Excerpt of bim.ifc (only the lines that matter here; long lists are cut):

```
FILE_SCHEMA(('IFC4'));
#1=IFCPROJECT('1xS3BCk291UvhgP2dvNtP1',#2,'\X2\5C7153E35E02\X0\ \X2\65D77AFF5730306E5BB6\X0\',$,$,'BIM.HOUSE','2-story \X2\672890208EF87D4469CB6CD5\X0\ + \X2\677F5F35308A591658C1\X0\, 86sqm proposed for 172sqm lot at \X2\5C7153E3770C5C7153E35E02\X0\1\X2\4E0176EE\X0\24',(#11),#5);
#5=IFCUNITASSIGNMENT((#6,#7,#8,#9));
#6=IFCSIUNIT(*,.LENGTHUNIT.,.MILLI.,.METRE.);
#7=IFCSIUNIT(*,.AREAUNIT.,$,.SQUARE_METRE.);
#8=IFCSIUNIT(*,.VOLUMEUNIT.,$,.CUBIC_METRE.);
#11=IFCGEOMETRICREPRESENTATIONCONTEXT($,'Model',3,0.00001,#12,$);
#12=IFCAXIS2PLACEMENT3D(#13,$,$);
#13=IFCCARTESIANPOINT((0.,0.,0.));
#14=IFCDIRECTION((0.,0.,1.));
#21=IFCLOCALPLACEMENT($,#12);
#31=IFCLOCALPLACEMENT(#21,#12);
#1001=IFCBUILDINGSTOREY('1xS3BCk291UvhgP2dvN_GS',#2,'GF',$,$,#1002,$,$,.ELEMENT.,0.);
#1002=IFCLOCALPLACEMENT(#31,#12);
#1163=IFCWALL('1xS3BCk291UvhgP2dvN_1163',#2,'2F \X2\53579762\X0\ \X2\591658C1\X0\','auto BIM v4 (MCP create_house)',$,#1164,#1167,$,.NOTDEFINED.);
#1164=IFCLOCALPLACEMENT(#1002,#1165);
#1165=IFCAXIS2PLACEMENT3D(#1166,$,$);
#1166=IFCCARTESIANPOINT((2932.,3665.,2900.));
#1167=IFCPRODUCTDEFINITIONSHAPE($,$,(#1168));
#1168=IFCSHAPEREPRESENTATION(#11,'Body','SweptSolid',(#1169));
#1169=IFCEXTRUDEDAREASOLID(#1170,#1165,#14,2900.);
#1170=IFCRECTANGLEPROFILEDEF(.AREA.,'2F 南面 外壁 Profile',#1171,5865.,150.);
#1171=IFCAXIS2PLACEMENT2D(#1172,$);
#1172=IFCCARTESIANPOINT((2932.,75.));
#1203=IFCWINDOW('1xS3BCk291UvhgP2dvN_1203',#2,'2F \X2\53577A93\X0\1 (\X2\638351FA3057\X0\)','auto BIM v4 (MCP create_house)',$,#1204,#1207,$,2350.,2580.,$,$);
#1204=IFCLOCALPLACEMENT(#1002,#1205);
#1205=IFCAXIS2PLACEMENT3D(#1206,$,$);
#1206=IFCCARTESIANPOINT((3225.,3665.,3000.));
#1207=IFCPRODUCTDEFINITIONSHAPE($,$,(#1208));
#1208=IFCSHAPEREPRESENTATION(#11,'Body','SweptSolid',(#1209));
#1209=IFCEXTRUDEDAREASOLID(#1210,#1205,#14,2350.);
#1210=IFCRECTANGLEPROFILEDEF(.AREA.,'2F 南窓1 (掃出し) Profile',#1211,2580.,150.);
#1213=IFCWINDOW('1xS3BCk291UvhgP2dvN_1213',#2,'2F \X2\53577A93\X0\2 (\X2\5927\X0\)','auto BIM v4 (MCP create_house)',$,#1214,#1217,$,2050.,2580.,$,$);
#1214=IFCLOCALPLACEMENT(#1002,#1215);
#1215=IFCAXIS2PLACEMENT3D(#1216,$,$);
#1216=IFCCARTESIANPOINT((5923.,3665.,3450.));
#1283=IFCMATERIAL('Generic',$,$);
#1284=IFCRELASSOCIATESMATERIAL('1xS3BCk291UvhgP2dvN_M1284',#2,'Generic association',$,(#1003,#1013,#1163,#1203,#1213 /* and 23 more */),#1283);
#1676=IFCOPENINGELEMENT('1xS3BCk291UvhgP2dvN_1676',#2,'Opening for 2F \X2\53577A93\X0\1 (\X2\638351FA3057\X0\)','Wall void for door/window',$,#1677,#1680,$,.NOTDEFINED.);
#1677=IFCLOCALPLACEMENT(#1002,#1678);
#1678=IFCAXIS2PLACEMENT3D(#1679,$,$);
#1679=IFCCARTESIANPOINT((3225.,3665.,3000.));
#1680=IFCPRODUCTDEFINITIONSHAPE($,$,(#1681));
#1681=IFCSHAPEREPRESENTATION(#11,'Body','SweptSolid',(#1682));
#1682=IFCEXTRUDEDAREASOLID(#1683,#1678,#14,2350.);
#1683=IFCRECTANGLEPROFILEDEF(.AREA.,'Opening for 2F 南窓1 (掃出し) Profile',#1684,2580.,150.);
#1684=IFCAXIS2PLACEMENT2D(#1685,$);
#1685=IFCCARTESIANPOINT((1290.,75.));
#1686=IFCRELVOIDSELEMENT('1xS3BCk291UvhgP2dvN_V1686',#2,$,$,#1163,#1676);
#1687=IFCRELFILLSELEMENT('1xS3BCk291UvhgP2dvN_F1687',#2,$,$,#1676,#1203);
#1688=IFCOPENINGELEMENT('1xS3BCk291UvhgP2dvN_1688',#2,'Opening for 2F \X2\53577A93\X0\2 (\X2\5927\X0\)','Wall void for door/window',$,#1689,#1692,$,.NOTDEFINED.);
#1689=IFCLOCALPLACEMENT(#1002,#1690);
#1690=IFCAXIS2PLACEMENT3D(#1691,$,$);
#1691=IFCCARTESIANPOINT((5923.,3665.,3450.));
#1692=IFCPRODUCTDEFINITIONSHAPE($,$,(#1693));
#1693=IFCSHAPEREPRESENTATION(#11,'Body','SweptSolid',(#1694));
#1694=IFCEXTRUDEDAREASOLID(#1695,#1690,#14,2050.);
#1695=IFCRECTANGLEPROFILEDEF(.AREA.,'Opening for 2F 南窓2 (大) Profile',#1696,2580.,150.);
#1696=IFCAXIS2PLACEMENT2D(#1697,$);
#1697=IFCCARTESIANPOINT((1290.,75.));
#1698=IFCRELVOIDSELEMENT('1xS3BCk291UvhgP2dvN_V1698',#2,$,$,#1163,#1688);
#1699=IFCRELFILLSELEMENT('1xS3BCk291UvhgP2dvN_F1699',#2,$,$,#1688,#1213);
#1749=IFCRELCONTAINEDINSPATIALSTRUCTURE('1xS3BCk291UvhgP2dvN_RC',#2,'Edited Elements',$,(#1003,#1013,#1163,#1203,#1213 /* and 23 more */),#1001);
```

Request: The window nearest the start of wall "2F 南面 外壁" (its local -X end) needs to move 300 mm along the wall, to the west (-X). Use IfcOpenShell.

```python
import ifcopenshell
import ifcopenshell.api.geometry
import ifcopenshell.util.placement
import ifcopenshell.util.unit

model = ifcopenshell.open("bim.ifc")
unit_scale = ifcopenshell.util.unit.calculate_unit_scale(model)

window = model.by_guid("1xS3BCk291UvhgP2dvN_1203")
opening = window.FillsVoids[0].RelatingOpeningElement
wall = opening.VoidsElements[0].RelatingBuildingElement

wall_matrix = ifcopenshell.util.placement.get_local_placement(wall.ObjectPlacement)
shift = wall_matrix[:3, 0] * -0.3 / unit_scale
before = ifcopenshell.util.placement.get_local_placement(window.ObjectPlacement)[:3, 3].copy()

# The window is not placed relative to its opening, so move both.
for product in (opening, window):
    matrix = ifcopenshell.util.placement.get_local_placement(product.ObjectPlacement)
    matrix[:3, 3] += shift
    ifcopenshell.api.geometry.edit_object_placement(model, product=product, matrix=matrix, is_si=False)

after = ifcopenshell.util.placement.get_local_placement(window.ObjectPlacement)[:3, 3]
print("window moved by", (after - before).round(3) + 0.0)

model.write("bim_updated.ifc")
```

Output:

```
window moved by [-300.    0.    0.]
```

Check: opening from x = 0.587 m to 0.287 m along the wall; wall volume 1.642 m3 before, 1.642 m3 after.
